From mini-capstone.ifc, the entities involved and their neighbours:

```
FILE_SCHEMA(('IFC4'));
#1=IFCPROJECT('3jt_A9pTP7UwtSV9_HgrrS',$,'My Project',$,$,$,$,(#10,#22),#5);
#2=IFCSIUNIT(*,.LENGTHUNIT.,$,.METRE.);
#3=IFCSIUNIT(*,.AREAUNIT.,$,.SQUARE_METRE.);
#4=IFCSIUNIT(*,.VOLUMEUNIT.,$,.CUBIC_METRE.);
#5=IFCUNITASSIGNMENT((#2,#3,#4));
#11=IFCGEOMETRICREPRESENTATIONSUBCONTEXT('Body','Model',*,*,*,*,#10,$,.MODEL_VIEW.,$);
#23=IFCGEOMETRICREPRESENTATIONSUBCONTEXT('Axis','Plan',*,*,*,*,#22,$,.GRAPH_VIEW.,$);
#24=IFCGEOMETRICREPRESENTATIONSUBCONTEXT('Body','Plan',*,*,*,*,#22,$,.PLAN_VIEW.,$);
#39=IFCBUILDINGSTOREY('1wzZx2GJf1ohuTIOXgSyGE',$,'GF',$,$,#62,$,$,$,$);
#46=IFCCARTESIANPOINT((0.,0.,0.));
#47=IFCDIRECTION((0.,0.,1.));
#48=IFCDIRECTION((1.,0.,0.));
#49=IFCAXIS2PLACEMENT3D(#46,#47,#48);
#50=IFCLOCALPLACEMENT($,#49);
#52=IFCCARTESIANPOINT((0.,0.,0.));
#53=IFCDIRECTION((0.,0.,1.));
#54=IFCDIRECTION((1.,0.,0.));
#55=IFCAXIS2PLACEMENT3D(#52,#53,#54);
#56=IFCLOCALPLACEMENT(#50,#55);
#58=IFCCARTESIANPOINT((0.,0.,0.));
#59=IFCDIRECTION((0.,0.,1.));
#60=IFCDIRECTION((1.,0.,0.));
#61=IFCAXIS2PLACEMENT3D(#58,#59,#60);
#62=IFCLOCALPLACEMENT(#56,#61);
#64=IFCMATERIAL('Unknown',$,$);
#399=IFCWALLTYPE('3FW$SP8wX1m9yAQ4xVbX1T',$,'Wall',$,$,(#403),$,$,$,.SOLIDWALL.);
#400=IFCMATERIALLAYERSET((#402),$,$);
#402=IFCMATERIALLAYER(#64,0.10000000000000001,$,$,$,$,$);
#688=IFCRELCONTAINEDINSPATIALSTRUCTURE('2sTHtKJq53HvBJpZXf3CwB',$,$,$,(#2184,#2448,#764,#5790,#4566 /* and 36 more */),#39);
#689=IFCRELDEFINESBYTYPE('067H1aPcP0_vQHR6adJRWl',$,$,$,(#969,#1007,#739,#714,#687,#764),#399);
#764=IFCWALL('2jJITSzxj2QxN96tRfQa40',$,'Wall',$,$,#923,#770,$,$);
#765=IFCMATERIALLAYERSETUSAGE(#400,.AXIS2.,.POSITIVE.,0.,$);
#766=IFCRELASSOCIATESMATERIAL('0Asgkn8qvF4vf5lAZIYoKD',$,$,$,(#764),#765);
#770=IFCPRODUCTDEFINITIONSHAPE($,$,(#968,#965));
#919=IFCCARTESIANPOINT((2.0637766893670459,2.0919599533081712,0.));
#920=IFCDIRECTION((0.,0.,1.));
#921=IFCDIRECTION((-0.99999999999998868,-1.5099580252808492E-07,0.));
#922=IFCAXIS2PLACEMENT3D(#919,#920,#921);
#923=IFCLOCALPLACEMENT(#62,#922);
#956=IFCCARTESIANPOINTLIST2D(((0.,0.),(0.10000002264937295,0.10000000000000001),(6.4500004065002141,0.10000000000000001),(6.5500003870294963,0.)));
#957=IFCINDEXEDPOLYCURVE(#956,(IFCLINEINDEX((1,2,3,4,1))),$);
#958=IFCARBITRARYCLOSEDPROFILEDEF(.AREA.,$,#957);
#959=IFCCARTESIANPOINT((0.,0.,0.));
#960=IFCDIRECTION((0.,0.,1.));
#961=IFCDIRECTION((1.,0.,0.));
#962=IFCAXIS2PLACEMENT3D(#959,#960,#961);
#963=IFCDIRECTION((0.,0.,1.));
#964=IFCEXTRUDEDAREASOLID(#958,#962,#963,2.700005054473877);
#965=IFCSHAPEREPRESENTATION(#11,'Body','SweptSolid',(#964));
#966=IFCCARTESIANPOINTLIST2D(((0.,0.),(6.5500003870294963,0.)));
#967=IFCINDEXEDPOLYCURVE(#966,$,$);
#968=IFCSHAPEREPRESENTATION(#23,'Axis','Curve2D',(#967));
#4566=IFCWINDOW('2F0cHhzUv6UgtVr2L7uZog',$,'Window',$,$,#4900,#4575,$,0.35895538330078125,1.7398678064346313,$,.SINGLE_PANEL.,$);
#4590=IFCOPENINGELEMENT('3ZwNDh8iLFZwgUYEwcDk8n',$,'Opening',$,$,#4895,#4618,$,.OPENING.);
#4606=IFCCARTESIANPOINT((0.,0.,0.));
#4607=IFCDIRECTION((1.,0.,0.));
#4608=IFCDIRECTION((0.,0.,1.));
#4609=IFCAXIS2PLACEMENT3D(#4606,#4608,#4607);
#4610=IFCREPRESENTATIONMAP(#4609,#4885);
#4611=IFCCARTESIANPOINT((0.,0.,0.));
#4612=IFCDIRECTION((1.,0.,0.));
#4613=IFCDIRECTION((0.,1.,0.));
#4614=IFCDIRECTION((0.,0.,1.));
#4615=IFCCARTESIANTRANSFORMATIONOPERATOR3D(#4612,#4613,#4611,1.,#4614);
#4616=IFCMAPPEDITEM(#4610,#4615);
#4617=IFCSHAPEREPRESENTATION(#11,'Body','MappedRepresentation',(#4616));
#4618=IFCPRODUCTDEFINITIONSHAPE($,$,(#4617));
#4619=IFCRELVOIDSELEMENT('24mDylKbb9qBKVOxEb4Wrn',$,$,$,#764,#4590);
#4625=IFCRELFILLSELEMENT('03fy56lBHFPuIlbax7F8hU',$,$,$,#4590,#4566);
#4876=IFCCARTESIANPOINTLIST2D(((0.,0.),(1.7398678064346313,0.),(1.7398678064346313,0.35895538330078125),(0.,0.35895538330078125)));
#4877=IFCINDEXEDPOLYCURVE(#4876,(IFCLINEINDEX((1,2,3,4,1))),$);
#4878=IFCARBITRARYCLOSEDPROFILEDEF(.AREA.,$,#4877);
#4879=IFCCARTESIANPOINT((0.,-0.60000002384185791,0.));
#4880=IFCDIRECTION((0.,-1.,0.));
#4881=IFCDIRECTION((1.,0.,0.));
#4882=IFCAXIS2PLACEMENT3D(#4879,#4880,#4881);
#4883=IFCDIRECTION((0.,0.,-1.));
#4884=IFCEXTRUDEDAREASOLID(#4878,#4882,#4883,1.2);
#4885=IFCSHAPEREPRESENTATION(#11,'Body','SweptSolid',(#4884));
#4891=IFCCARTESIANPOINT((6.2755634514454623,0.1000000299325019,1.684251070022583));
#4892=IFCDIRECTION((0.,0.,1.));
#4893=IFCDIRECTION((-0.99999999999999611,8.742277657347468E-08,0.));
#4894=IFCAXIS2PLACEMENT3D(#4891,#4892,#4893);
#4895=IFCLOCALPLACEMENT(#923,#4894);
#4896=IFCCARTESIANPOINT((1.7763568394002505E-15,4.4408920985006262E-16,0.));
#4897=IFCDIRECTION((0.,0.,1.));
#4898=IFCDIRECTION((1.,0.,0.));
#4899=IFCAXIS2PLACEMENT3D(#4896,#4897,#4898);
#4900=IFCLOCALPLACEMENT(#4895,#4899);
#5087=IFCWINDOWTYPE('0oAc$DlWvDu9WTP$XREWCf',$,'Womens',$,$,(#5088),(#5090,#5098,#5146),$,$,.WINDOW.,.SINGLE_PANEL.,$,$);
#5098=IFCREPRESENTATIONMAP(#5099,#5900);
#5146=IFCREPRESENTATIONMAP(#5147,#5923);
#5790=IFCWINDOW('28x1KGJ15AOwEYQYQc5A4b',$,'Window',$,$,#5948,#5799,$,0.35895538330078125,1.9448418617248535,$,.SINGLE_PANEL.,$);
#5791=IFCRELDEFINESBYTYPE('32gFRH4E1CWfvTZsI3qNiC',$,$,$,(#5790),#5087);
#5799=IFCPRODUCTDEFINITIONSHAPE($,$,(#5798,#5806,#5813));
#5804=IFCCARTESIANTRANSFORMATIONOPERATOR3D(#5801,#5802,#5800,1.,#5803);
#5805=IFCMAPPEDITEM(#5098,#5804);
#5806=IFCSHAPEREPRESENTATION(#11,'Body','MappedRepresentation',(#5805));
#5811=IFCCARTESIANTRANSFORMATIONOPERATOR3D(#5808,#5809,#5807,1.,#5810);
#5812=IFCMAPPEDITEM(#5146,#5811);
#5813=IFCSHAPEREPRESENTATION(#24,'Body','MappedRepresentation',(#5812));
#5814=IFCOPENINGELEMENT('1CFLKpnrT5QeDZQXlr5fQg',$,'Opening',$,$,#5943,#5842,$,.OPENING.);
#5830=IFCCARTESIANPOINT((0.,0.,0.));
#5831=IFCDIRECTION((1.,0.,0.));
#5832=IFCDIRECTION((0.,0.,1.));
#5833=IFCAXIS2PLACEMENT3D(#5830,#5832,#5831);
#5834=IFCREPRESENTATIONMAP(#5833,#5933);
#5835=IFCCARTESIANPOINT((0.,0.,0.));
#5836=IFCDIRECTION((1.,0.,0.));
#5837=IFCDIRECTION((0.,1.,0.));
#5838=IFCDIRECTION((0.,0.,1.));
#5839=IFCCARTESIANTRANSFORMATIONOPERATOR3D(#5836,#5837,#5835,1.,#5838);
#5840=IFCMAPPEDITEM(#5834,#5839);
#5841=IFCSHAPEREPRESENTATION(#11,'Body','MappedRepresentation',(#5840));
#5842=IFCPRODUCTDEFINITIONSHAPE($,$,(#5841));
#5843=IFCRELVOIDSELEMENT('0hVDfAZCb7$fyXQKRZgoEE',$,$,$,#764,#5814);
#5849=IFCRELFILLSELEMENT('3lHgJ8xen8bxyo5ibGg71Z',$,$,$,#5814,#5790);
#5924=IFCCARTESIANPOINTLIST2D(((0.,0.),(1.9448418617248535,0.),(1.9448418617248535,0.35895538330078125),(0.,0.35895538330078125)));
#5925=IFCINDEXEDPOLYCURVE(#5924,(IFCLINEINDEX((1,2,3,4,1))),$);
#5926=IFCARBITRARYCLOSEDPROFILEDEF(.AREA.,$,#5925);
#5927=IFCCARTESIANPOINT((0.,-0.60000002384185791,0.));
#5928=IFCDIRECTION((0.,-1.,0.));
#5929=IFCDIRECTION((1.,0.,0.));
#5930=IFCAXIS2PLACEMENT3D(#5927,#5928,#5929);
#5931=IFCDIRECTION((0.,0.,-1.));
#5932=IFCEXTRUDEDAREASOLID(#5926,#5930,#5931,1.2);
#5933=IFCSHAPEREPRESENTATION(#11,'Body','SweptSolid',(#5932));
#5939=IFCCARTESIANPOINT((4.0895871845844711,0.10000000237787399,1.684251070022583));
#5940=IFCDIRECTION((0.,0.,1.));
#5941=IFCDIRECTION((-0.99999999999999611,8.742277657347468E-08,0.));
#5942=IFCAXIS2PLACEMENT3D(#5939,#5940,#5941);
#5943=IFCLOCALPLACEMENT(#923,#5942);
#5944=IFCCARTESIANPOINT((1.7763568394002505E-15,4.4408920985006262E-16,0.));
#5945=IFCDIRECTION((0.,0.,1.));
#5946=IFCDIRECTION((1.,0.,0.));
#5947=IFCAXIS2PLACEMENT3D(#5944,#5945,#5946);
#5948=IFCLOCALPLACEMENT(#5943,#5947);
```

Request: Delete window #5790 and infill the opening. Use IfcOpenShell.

```python
import ifcopenshell
import ifcopenshell.api.feature
import ifcopenshell.api.root
import ifcopenshell.geom
import ifcopenshell.util.shape

model = ifcopenshell.open("mini-capstone.ifc")
settings = ifcopenshell.geom.settings()


def volume(element):
    """Net volume in cubic metres, openings subtracted."""
    shape = ifcopenshell.geom.create_shape(settings, element)
    return ifcopenshell.util.shape.get_volume(shape.geometry)


window = model.by_id(5790)
opening = window.FillsVoids[0].RelatingOpeningElement
wall = opening.VoidsElements[0].RelatingBuildingElement
before = volume(wall)

ifcopenshell.api.root.remove_product(model, product=window)
ifcopenshell.api.feature.remove_feature(model, feature=opening)

after = volume(wall)

print(f"wall volume {before:.3f} -> {after:.3f} m3")

model.write("mini-capstone_v2.ifc")
```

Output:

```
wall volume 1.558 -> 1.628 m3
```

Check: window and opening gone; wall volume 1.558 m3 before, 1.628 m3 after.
